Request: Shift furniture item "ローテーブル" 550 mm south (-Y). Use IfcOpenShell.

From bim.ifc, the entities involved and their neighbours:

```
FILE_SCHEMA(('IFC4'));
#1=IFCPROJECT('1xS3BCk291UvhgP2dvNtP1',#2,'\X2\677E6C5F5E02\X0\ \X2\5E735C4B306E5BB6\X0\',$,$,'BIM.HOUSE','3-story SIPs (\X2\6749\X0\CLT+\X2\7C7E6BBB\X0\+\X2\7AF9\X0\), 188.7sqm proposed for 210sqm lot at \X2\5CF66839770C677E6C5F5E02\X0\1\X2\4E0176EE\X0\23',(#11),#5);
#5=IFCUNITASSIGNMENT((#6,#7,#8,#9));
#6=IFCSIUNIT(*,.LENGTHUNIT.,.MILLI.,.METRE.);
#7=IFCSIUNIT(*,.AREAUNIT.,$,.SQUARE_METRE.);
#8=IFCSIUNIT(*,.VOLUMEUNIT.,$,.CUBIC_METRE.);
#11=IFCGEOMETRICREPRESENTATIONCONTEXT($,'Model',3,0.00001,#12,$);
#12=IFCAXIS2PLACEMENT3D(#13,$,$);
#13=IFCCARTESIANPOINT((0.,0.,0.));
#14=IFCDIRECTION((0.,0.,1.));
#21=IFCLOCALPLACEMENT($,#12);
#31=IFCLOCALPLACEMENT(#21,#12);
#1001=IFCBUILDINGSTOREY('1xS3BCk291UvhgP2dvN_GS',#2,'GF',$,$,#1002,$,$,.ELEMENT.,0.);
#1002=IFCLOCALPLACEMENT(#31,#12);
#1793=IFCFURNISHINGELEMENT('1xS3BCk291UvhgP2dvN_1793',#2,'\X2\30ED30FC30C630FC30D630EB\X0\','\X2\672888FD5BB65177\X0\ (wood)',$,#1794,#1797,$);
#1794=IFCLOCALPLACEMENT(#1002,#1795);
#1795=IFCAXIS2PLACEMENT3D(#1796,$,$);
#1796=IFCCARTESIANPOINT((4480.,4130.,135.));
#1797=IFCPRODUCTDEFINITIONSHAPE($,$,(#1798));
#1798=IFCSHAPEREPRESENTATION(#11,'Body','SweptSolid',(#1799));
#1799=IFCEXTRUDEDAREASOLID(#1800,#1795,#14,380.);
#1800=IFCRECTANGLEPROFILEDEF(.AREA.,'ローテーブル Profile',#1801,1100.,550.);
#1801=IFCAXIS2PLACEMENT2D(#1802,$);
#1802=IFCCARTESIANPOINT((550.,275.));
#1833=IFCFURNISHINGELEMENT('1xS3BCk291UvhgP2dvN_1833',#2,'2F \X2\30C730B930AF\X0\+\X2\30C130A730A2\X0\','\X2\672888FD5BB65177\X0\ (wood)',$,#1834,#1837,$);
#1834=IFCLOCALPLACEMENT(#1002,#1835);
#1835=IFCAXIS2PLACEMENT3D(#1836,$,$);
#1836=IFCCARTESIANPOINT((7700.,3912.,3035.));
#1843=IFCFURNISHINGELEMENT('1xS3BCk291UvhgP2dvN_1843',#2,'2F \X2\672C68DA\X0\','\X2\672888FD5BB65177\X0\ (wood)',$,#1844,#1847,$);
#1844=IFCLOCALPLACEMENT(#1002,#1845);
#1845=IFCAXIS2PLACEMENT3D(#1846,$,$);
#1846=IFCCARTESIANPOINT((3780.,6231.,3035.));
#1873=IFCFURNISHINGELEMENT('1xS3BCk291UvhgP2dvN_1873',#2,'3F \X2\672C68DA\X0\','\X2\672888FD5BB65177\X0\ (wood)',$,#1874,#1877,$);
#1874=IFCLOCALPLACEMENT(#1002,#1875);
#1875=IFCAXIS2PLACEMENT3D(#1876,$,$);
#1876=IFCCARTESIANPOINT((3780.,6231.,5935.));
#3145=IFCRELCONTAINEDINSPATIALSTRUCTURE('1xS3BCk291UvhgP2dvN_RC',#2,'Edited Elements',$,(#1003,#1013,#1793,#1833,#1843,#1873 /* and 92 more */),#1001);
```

```python
import ifcopenshell
import ifcopenshell.api.geometry
import ifcopenshell.util.placement

model = ifcopenshell.open("bim.ifc")

item = model.by_guid("1xS3BCk291UvhgP2dvN_1793")
matrix = ifcopenshell.util.placement.get_local_placement(item.ObjectPlacement)
matrix[1, 3] -= 550.0
ifcopenshell.api.geometry.edit_object_placement(model, product=item, matrix=matrix, is_si=False)

print(ifcopenshell.util.placement.get_local_placement(item.ObjectPlacement).round(3) + 0.0)

model.write("bim_v2.ifc")
```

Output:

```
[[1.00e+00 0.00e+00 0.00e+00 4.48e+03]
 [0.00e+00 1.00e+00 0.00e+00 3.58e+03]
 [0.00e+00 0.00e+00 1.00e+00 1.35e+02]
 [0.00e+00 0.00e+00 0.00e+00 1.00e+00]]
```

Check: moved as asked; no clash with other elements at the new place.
